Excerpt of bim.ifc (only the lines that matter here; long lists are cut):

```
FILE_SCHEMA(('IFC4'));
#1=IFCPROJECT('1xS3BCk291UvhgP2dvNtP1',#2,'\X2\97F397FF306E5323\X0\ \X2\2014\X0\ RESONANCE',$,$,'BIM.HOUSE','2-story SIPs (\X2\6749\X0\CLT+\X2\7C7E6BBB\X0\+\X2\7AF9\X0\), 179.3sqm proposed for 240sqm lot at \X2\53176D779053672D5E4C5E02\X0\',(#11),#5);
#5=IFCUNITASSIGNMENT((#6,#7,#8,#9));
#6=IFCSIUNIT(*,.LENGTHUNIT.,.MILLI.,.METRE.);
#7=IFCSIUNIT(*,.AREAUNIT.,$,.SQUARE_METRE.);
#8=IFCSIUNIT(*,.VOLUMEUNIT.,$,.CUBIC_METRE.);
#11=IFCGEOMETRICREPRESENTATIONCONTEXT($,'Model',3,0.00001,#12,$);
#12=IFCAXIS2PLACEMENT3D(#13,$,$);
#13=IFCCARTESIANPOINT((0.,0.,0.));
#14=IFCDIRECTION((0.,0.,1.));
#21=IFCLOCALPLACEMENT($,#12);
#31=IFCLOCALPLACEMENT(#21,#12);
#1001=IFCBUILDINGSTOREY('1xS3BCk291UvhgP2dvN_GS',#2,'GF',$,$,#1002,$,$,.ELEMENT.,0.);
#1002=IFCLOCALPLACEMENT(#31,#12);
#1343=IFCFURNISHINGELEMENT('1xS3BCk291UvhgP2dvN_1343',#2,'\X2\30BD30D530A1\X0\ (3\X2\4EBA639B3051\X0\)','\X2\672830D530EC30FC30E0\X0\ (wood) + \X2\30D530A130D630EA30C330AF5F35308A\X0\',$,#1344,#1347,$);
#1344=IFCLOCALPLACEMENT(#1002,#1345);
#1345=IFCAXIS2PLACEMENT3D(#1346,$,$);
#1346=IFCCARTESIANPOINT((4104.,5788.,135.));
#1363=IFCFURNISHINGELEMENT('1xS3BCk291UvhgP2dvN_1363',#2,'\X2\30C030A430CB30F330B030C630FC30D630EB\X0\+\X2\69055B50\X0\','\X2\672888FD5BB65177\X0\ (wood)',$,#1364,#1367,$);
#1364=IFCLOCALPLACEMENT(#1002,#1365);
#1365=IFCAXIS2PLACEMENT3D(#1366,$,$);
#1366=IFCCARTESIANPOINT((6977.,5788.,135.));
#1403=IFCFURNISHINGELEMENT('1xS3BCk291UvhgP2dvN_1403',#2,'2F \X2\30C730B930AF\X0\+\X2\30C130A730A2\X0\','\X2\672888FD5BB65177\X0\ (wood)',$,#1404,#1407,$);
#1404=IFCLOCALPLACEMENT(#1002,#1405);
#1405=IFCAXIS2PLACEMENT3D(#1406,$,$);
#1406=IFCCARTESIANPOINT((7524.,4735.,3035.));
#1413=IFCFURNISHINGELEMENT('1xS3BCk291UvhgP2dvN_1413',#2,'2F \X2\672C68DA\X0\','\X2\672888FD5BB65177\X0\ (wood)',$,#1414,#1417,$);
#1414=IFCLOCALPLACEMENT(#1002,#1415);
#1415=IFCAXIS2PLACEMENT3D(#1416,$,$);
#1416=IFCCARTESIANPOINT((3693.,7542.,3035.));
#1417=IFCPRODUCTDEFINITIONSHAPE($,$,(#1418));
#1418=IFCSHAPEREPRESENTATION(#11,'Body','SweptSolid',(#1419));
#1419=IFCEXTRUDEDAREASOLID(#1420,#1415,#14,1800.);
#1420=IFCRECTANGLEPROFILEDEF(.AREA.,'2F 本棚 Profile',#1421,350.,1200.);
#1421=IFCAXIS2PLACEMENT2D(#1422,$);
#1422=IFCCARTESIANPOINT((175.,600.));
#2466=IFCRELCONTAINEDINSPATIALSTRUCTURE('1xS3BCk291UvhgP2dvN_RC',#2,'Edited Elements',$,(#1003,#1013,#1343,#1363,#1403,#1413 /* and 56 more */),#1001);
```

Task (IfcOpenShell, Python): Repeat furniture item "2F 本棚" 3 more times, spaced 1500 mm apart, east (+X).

```python
import numpy as np
import ifcopenshell
import ifcopenshell.api.geometry
import ifcopenshell.api.root
import ifcopenshell.util.element
import ifcopenshell.util.placement
import ifcopenshell.util.unit

model = ifcopenshell.open("bim.ifc")
unit_scale = ifcopenshell.util.unit.calculate_unit_scale(model)


def reuse_history(source, copy):
    """copy_class also copies each property set's owner history, people and application; keep the originals."""
    for rel in copy.IsDefinedBy:
        if rel.is_a("IfcRelDefinesByProperties") and (history := rel.RelatingPropertyDefinition.OwnerHistory):
            rel.RelatingPropertyDefinition.OwnerHistory = source.OwnerHistory
            ifcopenshell.util.element.remove_deep2(model, history)


source = model.by_guid("1xS3BCk291UvhgP2dvN_1413")
base = ifcopenshell.util.placement.get_local_placement(source.ObjectPlacement)
step = np.array([1.0, 0.0, 0.0]) * 1.5 / unit_scale

for i in range(1, 4):
    copy = ifcopenshell.api.root.copy_class(model, product=source)
    copy.Representation = ifcopenshell.util.element.copy_deep(
        model, source.Representation, exclude=["IfcGeometricRepresentationContext", "IfcRepresentationMap"]
    )
    reuse_history(source, copy)
    matrix = base.copy()
    matrix[:3, 3] += i * step
    print("added at", matrix[:3, 3].round(3) + 0.0)
    ifcopenshell.api.geometry.edit_object_placement(model, product=copy, matrix=matrix, is_si=False)

model.write("bim_rev.ifc")
```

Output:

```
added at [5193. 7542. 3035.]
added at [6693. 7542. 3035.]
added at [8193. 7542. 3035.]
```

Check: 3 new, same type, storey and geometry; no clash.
